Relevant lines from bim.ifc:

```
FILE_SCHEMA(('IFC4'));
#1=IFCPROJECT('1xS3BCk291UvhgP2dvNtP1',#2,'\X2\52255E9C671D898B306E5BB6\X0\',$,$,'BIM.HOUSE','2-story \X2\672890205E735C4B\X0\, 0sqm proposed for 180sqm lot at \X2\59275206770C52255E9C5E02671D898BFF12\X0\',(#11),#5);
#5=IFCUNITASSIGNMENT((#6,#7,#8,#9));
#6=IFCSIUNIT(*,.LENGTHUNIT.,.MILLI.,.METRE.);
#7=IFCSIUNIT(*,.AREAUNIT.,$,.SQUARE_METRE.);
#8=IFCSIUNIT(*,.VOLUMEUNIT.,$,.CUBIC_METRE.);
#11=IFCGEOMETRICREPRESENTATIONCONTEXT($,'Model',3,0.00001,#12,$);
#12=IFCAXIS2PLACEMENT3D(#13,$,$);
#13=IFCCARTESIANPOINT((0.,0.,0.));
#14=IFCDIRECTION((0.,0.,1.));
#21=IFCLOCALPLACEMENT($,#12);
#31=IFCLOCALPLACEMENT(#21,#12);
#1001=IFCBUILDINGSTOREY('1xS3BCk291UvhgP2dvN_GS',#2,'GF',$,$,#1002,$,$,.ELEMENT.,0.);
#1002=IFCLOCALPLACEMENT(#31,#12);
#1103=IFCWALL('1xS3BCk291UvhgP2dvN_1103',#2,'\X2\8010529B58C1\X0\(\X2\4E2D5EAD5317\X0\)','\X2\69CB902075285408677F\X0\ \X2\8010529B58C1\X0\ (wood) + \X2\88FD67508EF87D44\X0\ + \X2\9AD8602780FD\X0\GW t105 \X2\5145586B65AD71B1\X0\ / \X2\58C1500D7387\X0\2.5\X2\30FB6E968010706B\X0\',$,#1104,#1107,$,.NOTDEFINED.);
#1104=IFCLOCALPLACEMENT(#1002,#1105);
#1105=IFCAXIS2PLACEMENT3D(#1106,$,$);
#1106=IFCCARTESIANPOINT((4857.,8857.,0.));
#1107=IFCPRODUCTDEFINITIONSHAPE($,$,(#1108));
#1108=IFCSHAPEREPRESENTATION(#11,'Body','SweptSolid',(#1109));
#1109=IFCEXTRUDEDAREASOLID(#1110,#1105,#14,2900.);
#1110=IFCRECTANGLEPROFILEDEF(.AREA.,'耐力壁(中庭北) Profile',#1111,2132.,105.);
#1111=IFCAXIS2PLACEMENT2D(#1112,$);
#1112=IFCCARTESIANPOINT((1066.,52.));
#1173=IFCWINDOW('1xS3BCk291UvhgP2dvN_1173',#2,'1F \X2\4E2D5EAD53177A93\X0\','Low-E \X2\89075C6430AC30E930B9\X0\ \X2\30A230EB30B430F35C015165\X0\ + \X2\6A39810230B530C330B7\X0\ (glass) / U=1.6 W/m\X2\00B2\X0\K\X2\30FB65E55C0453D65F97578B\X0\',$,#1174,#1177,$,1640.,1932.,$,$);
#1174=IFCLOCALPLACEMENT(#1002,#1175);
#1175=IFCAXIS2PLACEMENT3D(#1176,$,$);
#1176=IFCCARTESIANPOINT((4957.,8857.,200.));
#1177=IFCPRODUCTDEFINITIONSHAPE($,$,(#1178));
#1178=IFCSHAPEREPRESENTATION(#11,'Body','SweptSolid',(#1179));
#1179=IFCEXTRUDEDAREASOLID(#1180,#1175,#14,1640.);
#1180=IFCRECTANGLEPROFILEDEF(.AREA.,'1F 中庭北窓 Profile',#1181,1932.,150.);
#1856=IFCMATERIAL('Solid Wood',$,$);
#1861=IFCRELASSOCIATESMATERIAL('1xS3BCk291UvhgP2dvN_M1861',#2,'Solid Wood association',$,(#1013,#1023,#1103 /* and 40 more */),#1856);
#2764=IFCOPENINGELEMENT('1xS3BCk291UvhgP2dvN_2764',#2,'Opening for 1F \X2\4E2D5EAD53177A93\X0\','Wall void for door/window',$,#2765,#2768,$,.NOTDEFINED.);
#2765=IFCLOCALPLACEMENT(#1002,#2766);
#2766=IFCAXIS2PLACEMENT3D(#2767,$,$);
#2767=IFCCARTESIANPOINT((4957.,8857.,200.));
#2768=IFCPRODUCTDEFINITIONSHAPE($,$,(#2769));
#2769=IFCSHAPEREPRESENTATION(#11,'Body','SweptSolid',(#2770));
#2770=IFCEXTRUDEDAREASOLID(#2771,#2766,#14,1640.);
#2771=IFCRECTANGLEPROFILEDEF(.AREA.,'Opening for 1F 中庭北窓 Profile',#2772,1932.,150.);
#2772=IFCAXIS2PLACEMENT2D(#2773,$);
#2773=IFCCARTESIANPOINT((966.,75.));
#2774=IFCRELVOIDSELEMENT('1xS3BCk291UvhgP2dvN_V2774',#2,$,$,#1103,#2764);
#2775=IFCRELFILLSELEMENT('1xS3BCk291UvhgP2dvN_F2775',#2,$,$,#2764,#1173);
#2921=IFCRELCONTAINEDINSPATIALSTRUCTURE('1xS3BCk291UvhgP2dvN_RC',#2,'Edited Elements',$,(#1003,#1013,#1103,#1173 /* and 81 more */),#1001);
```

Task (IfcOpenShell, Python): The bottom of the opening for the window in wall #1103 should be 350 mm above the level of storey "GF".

```python
import numpy as np
import ifcopenshell
import ifcopenshell.api.geometry
import ifcopenshell.geom
import ifcopenshell.util.element
import ifcopenshell.util.placement
import ifcopenshell.util.shape
import ifcopenshell.util.unit

model = ifcopenshell.open("bim.ifc")
unit_scale = ifcopenshell.util.unit.calculate_unit_scale(model)

window = model.by_guid("1xS3BCk291UvhgP2dvN_1173")
opening = window.FillsVoids[0].RelatingOpeningElement
storey = ifcopenshell.util.element.get_container(window, ifc_class="IfcBuildingStorey")
level = ifcopenshell.util.placement.get_local_placement(storey.ObjectPlacement)[2, 3]

# The opening's origin need not be at the sill, so measure its lowest point.
shape = ifcopenshell.geom.create_shape(ifcopenshell.geom.settings(), opening)
bottom = ifcopenshell.util.shape.get_shape_bottom_elevation(shape, shape.geometry) / unit_scale
dz = level + 350.0 - bottom

shift = np.array([0.0, 0.0, dz])
# The window is not placed relative to its opening, so move both.
for product in (opening, window):
    matrix = ifcopenshell.util.placement.get_local_placement(product.ObjectPlacement)
    matrix[:3, 3] += shift
    ifcopenshell.api.geometry.edit_object_placement(model, product=product, matrix=matrix, is_si=False)

print(f"moved by {dz * unit_scale:+.3f} m")

model.write("bim_updated.ifc")
```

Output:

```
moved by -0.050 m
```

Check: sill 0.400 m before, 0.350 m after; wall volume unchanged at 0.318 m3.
